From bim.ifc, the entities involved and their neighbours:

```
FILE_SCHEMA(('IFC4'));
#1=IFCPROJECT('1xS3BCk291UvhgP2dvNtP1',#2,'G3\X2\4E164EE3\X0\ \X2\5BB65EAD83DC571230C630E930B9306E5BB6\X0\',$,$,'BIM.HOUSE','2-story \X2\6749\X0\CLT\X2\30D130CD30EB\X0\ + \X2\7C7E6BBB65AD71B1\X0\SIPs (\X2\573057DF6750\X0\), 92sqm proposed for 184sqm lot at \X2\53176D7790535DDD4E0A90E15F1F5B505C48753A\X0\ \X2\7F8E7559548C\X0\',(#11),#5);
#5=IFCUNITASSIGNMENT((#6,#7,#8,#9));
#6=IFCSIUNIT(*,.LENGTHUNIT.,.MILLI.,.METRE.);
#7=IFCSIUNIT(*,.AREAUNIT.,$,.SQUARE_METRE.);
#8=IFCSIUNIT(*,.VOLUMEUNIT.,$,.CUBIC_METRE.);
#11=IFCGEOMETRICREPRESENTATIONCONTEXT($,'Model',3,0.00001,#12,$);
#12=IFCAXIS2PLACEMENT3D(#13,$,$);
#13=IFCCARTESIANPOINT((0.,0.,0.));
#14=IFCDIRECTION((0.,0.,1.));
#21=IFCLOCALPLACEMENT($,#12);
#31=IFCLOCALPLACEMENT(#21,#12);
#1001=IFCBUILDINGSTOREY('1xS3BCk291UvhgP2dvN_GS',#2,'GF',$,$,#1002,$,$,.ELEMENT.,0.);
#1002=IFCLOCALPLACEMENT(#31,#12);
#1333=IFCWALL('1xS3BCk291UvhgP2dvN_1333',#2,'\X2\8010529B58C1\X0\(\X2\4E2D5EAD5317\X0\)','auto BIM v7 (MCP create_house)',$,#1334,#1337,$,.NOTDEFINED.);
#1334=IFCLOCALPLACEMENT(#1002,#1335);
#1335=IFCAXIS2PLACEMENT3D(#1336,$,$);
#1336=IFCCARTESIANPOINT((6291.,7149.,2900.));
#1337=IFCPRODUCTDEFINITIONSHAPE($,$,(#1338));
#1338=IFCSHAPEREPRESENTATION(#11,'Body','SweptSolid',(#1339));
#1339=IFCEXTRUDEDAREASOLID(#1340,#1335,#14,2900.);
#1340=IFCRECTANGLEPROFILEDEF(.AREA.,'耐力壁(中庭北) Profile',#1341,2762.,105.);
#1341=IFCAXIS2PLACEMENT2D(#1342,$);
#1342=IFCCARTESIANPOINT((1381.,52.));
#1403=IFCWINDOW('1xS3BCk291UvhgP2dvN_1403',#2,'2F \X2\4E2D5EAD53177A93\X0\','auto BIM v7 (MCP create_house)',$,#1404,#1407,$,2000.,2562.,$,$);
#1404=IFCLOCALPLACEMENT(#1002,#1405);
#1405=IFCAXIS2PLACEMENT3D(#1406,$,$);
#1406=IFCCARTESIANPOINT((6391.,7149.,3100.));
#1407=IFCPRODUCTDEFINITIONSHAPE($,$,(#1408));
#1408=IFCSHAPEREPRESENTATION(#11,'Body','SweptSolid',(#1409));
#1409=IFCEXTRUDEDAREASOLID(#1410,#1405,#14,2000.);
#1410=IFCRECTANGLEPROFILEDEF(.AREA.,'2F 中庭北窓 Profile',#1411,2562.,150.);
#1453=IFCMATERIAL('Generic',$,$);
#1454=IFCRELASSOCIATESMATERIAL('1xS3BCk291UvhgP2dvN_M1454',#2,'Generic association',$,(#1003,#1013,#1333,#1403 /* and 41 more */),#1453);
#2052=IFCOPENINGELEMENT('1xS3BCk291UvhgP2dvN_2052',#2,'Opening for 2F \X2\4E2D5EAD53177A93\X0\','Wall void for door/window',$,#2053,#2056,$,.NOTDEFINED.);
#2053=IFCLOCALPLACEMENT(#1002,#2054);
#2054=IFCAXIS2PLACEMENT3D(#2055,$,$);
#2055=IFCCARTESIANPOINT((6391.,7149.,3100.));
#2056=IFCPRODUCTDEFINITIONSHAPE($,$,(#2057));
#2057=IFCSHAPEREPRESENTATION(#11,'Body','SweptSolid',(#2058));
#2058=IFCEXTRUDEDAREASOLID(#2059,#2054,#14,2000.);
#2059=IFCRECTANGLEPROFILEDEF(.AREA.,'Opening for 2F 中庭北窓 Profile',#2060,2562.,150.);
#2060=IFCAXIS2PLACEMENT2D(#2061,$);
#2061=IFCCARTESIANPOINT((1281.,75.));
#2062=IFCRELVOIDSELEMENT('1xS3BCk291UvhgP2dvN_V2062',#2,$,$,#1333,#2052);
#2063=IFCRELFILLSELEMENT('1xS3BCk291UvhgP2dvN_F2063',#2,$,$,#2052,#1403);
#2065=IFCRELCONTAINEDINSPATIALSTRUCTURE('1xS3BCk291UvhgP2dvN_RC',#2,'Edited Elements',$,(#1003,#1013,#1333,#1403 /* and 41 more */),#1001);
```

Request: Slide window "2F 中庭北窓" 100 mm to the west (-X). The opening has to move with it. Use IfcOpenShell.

```python
import ifcopenshell
import ifcopenshell.api.geometry
import ifcopenshell.util.placement
import ifcopenshell.util.unit

model = ifcopenshell.open("bim.ifc")
unit_scale = ifcopenshell.util.unit.calculate_unit_scale(model)

window = model.by_guid("1xS3BCk291UvhgP2dvN_1403")
opening = window.FillsVoids[0].RelatingOpeningElement
wall = opening.VoidsElements[0].RelatingBuildingElement

wall_matrix = ifcopenshell.util.placement.get_local_placement(wall.ObjectPlacement)
shift = wall_matrix[:3, 0] * -0.1 / unit_scale
before = ifcopenshell.util.placement.get_local_placement(window.ObjectPlacement)[:3, 3].copy()

# The window is not placed relative to its opening, so move both.
for product in (opening, window):
    matrix = ifcopenshell.util.placement.get_local_placement(product.ObjectPlacement)
    matrix[:3, 3] += shift
    ifcopenshell.api.geometry.edit_object_placement(model, product=product, matrix=matrix, is_si=False)

after = ifcopenshell.util.placement.get_local_placement(window.ObjectPlacement)[:3, 3]
print("window moved by", (after - before).round(3) + 0.0)

model.write("bim_v2.ifc")
```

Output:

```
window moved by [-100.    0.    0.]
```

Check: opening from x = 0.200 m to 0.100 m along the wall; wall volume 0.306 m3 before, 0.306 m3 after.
